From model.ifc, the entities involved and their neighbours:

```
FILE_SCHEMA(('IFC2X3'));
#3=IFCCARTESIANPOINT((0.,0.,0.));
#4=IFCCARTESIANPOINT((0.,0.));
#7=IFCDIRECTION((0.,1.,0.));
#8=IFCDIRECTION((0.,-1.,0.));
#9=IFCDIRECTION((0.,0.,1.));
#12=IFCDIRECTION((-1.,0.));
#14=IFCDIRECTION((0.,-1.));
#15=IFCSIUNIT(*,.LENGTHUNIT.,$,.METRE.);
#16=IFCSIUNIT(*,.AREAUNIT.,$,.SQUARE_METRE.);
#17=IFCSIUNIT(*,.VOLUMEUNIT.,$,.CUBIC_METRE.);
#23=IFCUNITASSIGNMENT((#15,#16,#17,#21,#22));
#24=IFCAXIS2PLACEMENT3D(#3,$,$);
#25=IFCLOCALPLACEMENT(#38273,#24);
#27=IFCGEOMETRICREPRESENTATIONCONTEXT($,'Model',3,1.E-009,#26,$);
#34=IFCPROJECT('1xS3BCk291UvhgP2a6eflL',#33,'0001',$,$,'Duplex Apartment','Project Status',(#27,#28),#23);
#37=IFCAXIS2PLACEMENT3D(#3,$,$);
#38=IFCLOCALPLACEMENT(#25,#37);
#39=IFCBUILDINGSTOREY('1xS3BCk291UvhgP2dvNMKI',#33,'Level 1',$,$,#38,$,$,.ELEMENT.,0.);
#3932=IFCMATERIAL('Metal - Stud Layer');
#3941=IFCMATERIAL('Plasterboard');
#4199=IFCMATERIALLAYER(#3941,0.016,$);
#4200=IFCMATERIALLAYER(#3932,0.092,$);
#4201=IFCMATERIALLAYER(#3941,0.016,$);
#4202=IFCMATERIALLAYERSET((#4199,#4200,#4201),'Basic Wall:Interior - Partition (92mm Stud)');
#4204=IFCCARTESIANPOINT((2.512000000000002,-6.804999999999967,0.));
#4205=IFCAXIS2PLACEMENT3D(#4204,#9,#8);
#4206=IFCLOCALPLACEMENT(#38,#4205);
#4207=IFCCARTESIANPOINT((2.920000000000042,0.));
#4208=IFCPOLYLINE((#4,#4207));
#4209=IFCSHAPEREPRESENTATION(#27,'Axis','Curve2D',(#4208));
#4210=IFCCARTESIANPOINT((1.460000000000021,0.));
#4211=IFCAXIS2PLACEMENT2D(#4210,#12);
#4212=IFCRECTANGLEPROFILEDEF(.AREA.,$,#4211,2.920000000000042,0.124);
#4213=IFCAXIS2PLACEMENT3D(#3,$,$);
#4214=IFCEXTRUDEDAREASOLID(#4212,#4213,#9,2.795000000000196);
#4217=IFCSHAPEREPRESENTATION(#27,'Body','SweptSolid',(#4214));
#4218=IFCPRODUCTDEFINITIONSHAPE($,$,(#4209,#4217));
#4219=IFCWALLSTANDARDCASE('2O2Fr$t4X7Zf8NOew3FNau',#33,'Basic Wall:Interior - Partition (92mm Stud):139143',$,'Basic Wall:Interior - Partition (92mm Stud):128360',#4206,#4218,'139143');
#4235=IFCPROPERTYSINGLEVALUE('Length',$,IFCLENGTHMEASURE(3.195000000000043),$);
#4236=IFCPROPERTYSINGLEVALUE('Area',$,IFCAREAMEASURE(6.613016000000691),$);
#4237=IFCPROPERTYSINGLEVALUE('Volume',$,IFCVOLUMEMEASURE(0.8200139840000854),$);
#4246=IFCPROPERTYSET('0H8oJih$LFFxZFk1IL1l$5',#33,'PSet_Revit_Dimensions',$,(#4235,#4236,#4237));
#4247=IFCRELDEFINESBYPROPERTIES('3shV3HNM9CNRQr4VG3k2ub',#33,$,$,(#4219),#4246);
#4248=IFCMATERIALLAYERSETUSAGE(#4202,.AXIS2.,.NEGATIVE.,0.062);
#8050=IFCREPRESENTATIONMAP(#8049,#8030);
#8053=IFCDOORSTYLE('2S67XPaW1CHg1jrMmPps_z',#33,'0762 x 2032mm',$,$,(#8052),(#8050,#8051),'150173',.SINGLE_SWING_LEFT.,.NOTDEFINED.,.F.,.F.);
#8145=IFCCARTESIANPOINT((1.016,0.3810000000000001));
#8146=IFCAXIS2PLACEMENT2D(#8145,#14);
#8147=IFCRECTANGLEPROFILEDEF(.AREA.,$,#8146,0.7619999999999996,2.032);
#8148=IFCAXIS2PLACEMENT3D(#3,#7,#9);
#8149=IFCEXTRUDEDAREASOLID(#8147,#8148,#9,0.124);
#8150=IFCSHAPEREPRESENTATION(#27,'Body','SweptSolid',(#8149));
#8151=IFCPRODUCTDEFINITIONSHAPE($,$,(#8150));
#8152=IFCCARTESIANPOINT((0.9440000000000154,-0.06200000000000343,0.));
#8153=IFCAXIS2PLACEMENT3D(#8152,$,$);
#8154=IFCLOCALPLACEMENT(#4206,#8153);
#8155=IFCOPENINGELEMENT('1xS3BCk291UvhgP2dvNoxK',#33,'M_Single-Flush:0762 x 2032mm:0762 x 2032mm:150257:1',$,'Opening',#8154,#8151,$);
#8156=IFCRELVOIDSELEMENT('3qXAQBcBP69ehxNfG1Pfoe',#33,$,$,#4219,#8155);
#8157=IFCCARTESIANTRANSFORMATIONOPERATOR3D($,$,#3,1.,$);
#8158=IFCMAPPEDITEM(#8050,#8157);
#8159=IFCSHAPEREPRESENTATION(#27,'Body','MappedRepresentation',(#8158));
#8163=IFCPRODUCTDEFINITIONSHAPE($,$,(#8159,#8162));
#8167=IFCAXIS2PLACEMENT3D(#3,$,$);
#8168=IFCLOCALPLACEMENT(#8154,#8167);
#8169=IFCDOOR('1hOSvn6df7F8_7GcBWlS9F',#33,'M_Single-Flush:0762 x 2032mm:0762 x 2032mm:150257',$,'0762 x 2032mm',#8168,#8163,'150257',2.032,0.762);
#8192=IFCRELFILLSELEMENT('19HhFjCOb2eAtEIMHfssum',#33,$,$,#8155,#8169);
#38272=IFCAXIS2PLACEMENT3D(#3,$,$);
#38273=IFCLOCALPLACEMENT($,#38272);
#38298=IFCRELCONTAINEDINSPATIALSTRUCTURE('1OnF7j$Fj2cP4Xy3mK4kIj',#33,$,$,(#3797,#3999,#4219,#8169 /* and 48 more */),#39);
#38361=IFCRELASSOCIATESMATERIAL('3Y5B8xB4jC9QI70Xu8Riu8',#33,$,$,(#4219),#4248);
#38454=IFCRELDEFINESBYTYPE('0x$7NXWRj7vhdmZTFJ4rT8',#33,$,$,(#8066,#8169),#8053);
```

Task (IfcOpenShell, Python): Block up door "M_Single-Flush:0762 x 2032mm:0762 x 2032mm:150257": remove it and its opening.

```python
import ifcopenshell
import ifcopenshell.api.feature
import ifcopenshell.api.pset
import ifcopenshell.api.root
import ifcopenshell.geom
import ifcopenshell.util.element
import ifcopenshell.util.shape
import ifcopenshell.util.unit

model = ifcopenshell.open("model.ifc")
area_scale = ifcopenshell.util.unit.calculate_unit_scale(model, "AREAUNIT")
volume_scale = ifcopenshell.util.unit.calculate_unit_scale(model, "VOLUMEUNIT")
settings = ifcopenshell.geom.settings()


def volume(element):
    """Net volume in cubic metres, openings subtracted."""
    shape = ifcopenshell.geom.create_shape(settings, element)
    return ifcopenshell.util.shape.get_volume(shape.geometry)


door = model.by_guid("1hOSvn6df7F8_7GcBWlS9F")
opening = door.FillsVoids[0].RelatingOpeningElement
wall = opening.VoidsElements[0].RelatingBuildingElement
before = volume(wall)

ifcopenshell.api.root.remove_product(model, product=door)
ifcopenshell.api.feature.remove_feature(model, feature=opening)

after = volume(wall)
thickness = 0.124  # wall thickness in metres

# Update the wall's stored quantities.
pset = model.by_id(ifcopenshell.util.element.get_pset(wall, "PSet_Revit_Dimensions", should_inherit=False)["id"])
ifcopenshell.api.pset.edit_pset(model, pset=pset, properties={
    "Area": model.create_entity("IfcAreaMeasure", after / thickness / area_scale),
    "Volume": model.create_entity("IfcVolumeMeasure", after / volume_scale),
})

print(f"wall volume {before:.3f} -> {after:.3f} m3")

model.write("model-out.ifc")
```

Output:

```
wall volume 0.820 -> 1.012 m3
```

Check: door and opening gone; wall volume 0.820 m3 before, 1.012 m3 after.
